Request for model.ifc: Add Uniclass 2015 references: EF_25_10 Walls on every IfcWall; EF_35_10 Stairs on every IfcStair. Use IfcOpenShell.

First a look at what the model holds.

```python
import ifcopenshell

model = ifcopenshell.open("model.ifc")
print(model.schema)
print("classifications:", [c.Name for c in model.by_type("IfcClassification")])
for ifc_class in ("IfcDoor", "IfcRoof", "IfcStair", "IfcWall", "IfcWindow"):
    print(ifc_class, len(model.by_type(ifc_class)))
```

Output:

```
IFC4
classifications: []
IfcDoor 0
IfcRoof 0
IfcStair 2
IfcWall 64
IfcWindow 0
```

```python
import ifcopenshell
import ifcopenshell.api.classification

model = ifcopenshell.open("model.ifc")

system = ifcopenshell.api.classification.add_classification(model, classification="Uniclass 2015")

codes = {
    "IfcWall": ("EF_25_10", "Walls"),
    "IfcStair": ("EF_35_10", "Stairs"),
}
for ifc_class, (code, name) in codes.items():
    products = model.by_type(ifc_class)
    ifcopenshell.api.classification.add_reference(
        model, products=products, classification=system, identification=code, name=name
    )
    print(code, len(products))

model.write("model_rev.ifc")
```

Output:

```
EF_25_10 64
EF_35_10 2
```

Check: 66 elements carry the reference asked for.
